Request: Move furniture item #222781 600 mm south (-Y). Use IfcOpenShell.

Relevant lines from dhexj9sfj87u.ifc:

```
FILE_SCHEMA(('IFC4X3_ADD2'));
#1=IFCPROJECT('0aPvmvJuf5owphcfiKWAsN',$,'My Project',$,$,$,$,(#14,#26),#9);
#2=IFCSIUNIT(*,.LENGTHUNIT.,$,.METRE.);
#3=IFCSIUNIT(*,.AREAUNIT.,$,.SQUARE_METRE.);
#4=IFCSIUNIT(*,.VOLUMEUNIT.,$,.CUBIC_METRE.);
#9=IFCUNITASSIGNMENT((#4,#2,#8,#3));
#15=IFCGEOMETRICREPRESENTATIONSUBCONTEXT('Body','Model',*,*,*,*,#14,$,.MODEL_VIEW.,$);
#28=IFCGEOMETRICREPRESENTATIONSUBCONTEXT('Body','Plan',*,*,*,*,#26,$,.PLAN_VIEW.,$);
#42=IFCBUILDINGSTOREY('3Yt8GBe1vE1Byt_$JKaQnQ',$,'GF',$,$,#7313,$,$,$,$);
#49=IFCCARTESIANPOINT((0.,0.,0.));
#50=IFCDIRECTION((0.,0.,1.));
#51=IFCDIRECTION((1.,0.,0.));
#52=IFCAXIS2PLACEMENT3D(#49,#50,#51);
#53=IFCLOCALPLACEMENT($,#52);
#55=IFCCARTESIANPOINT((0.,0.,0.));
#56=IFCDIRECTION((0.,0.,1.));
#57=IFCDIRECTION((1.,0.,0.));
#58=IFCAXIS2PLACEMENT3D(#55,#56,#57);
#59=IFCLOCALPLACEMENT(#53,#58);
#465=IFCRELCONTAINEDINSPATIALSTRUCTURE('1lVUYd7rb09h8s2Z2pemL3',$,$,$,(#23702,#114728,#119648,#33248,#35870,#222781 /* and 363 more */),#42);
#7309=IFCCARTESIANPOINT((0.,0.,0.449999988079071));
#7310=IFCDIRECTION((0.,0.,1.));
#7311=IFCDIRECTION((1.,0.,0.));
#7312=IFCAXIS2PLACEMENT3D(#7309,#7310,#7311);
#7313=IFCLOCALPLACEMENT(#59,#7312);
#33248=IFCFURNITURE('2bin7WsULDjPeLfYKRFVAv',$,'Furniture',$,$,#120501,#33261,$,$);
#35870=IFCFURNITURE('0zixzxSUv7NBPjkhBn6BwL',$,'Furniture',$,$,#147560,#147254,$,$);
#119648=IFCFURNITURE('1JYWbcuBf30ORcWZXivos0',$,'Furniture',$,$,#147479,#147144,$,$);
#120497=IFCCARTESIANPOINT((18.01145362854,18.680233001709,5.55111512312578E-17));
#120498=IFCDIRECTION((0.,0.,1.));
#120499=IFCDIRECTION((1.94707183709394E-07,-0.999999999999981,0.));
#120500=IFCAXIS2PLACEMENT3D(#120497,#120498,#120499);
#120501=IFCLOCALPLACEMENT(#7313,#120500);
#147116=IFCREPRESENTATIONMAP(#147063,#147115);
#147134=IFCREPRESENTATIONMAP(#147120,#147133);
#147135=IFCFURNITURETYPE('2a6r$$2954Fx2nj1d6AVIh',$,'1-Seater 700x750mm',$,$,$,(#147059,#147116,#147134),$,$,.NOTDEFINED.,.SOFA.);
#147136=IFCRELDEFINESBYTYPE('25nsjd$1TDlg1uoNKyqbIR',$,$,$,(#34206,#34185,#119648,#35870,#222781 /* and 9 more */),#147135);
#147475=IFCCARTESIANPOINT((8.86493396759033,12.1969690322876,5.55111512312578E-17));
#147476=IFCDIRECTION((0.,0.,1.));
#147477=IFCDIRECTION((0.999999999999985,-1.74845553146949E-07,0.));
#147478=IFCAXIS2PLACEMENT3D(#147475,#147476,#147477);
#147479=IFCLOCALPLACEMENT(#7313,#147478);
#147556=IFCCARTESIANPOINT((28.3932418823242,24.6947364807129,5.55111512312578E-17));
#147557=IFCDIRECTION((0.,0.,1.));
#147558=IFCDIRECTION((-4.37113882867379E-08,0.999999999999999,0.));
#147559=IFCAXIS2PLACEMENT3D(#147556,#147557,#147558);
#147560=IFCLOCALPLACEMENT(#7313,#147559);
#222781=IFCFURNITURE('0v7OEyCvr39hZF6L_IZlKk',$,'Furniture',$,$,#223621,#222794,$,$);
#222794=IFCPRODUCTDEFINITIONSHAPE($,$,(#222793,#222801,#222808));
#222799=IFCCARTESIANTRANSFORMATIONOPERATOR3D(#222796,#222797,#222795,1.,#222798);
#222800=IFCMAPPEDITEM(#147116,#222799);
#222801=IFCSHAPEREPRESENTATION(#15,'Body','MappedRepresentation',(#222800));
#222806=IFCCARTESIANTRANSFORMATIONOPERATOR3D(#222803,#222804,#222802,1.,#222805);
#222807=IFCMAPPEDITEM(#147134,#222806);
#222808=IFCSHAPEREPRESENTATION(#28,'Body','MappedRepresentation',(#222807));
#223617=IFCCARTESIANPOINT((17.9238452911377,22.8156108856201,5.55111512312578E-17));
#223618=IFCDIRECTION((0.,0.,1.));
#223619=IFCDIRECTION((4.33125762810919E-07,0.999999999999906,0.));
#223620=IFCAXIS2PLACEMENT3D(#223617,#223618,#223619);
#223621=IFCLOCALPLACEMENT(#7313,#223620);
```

```python
import ifcopenshell
import ifcopenshell.api.geometry
import ifcopenshell.util.placement
import ifcopenshell.util.unit

model = ifcopenshell.open("dhexj9sfj87u.ifc")
unit_scale = ifcopenshell.util.unit.calculate_unit_scale(model)

item = model.by_id(222781)
matrix = ifcopenshell.util.placement.get_local_placement(item.ObjectPlacement)
matrix[1, 3] -= 0.6 / unit_scale
ifcopenshell.api.geometry.edit_object_placement(model, product=item, matrix=matrix, is_si=False)

print(ifcopenshell.util.placement.get_local_placement(item.ObjectPlacement).round(3) + 0.0)

model.write("dhexj9sfj87u_v2.ifc")
```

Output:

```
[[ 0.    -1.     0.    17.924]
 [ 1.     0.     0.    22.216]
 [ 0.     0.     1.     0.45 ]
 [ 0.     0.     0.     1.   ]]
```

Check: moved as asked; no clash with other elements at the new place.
